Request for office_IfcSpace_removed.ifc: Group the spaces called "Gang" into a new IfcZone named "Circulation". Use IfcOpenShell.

First a look at what the model holds.

```python
import ifcopenshell

model = ifcopenshell.open("office_IfcSpace_removed.ifc")
print(model.schema)
seen = {}
for space in model.by_type("IfcSpace"):
    seen[space.LongName] = seen.get(space.LongName, 0) + 1
for name, count in sorted(seen.items(), key=str):
    print(count, "x", name)
print("zones:", [z.Name for z in model.by_type("IfcZone")][:20])
```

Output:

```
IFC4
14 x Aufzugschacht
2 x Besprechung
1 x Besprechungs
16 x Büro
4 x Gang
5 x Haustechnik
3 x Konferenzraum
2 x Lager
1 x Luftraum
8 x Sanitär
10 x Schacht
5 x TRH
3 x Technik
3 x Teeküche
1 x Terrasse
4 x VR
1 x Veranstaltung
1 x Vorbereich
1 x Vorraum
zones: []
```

```python
import ifcopenshell
import ifcopenshell.api.group
import ifcopenshell.api.root

model = ifcopenshell.open("office_IfcSpace_removed.ifc")

names = {"Gang"}
spaces = [s for s in model.by_type("IfcSpace") if s.LongName in names]

zone = ifcopenshell.api.root.create_entity(model, ifc_class="IfcZone", name="Circulation")
ifcopenshell.api.group.assign_group(model, products=spaces, group=zone)
print(len(spaces), "spaces in", zone.Name)

model.write("office_IfcSpace_removed_updated.ifc")
```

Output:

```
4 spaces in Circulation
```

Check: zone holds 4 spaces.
